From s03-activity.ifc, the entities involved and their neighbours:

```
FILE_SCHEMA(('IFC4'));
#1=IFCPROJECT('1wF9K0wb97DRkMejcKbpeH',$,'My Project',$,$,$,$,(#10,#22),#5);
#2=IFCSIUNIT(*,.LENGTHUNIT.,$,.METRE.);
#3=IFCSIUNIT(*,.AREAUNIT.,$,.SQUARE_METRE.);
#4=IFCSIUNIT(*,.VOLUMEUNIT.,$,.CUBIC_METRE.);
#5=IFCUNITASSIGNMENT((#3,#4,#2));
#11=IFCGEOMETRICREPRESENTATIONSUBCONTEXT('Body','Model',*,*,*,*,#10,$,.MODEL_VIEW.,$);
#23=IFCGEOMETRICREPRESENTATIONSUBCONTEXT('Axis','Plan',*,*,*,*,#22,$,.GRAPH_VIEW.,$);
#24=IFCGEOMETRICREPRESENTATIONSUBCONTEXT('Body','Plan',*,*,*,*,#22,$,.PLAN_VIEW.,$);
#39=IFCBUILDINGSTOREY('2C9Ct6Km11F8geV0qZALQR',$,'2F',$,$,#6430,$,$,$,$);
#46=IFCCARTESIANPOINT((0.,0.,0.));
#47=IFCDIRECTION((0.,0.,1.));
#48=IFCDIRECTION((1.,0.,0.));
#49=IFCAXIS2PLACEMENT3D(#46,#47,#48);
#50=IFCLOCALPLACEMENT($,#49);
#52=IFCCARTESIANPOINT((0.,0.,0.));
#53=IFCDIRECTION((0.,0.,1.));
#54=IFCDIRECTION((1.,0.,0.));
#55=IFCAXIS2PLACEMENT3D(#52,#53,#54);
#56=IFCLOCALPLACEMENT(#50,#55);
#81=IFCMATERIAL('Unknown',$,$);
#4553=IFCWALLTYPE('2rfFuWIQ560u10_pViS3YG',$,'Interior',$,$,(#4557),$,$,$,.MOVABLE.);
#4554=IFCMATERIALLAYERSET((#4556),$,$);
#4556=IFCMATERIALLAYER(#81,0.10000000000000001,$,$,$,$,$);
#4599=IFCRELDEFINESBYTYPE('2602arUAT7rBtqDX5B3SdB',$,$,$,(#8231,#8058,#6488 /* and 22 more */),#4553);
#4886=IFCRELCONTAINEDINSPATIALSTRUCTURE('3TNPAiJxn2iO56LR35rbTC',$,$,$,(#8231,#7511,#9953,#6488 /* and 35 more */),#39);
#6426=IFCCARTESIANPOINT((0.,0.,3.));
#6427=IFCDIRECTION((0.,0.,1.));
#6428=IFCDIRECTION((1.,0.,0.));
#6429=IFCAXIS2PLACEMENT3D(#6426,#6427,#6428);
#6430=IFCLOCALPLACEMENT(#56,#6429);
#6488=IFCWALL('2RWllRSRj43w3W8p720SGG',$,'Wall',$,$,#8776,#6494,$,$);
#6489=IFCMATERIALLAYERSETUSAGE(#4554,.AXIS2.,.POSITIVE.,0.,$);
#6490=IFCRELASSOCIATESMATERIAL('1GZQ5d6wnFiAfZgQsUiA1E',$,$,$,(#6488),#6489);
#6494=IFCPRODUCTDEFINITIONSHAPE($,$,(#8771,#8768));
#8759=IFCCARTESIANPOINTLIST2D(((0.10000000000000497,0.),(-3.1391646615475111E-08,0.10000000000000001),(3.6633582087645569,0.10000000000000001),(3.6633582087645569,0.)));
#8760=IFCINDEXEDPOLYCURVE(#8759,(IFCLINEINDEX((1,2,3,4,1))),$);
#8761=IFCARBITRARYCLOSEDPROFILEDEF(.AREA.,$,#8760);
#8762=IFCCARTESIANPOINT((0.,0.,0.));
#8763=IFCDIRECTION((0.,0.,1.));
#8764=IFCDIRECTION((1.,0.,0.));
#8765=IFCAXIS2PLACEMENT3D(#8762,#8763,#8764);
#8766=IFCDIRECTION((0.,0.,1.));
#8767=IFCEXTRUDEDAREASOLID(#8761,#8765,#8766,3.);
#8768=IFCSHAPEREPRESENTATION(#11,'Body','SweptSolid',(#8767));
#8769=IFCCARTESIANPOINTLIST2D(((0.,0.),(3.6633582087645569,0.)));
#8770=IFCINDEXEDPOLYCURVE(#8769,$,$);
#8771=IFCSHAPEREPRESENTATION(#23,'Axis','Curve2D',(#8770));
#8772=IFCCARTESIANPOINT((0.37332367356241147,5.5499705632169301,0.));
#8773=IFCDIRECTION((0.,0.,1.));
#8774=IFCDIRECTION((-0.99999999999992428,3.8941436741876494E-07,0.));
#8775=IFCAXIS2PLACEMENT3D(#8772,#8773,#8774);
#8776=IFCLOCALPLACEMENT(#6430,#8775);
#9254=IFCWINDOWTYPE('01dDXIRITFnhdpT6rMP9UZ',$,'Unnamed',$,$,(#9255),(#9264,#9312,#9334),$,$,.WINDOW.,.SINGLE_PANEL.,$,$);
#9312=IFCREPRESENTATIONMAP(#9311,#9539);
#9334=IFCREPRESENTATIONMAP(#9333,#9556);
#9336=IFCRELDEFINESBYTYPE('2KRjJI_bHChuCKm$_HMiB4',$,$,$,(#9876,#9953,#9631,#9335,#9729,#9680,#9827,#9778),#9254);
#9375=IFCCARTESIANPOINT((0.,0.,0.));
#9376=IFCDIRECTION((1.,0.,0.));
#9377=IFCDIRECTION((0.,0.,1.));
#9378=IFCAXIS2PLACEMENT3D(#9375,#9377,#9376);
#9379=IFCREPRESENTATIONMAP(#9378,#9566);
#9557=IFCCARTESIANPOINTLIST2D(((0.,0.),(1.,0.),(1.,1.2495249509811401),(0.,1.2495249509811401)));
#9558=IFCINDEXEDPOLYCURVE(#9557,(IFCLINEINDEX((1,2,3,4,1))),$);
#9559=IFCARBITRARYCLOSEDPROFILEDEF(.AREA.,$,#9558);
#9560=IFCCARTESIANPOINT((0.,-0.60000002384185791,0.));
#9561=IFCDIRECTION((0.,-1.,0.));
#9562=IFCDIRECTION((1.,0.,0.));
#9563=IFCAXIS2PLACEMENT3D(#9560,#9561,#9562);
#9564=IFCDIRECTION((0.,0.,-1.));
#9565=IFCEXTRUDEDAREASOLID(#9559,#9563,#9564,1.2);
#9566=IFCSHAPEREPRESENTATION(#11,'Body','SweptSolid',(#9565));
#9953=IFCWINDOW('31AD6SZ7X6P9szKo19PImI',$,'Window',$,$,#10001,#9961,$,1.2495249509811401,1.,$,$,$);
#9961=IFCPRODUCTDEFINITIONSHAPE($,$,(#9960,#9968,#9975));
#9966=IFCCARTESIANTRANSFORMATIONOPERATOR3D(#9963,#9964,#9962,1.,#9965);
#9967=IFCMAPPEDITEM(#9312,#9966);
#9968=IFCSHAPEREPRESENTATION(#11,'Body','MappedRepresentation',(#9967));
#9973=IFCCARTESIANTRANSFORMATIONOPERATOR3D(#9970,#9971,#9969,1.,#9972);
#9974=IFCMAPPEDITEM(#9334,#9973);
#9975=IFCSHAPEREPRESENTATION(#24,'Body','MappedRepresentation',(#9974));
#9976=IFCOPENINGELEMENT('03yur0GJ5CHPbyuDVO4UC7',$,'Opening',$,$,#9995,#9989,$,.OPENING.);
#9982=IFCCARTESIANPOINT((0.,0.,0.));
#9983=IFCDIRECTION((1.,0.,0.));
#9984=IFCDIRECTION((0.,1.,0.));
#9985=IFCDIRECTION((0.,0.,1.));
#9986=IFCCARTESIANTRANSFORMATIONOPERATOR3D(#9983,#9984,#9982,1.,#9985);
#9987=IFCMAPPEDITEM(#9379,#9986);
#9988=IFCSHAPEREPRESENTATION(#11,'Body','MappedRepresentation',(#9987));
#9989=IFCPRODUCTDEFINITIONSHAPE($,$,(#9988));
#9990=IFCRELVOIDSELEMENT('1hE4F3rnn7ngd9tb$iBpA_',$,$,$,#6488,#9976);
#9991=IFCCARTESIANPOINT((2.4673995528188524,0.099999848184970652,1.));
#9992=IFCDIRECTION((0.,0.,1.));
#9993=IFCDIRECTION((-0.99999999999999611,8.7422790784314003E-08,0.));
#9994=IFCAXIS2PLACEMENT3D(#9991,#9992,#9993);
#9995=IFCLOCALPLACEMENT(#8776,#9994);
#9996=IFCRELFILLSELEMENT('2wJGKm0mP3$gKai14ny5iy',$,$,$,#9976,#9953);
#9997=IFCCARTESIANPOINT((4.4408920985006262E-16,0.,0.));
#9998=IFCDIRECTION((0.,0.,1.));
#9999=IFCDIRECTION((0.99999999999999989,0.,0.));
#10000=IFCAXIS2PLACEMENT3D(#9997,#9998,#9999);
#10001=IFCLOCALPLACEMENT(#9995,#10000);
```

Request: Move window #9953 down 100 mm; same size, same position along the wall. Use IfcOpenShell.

```python
import numpy as np
import ifcopenshell
import ifcopenshell.api.geometry
import ifcopenshell.util.placement
import ifcopenshell.util.unit

model = ifcopenshell.open("s03-activity.ifc")
unit_scale = ifcopenshell.util.unit.calculate_unit_scale(model)

window = model.by_guid("31AD6SZ7X6P9szKo19PImI")
opening = window.FillsVoids[0].RelatingOpeningElement
dz = -0.1

shift = np.array([0.0, 0.0, dz])
# The window is placed relative to its opening, so it follows when the opening moves.
matrix = ifcopenshell.util.placement.get_local_placement(opening.ObjectPlacement)
matrix[:3, 3] += shift
ifcopenshell.api.geometry.edit_object_placement(
    model, product=opening, matrix=matrix, is_si=False, should_transform_children=True
)

print(f"moved by {dz * unit_scale:+.3f} m")

model.write("s03-activity_edited.ifc")
```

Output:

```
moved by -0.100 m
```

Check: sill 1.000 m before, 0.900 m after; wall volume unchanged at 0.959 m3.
